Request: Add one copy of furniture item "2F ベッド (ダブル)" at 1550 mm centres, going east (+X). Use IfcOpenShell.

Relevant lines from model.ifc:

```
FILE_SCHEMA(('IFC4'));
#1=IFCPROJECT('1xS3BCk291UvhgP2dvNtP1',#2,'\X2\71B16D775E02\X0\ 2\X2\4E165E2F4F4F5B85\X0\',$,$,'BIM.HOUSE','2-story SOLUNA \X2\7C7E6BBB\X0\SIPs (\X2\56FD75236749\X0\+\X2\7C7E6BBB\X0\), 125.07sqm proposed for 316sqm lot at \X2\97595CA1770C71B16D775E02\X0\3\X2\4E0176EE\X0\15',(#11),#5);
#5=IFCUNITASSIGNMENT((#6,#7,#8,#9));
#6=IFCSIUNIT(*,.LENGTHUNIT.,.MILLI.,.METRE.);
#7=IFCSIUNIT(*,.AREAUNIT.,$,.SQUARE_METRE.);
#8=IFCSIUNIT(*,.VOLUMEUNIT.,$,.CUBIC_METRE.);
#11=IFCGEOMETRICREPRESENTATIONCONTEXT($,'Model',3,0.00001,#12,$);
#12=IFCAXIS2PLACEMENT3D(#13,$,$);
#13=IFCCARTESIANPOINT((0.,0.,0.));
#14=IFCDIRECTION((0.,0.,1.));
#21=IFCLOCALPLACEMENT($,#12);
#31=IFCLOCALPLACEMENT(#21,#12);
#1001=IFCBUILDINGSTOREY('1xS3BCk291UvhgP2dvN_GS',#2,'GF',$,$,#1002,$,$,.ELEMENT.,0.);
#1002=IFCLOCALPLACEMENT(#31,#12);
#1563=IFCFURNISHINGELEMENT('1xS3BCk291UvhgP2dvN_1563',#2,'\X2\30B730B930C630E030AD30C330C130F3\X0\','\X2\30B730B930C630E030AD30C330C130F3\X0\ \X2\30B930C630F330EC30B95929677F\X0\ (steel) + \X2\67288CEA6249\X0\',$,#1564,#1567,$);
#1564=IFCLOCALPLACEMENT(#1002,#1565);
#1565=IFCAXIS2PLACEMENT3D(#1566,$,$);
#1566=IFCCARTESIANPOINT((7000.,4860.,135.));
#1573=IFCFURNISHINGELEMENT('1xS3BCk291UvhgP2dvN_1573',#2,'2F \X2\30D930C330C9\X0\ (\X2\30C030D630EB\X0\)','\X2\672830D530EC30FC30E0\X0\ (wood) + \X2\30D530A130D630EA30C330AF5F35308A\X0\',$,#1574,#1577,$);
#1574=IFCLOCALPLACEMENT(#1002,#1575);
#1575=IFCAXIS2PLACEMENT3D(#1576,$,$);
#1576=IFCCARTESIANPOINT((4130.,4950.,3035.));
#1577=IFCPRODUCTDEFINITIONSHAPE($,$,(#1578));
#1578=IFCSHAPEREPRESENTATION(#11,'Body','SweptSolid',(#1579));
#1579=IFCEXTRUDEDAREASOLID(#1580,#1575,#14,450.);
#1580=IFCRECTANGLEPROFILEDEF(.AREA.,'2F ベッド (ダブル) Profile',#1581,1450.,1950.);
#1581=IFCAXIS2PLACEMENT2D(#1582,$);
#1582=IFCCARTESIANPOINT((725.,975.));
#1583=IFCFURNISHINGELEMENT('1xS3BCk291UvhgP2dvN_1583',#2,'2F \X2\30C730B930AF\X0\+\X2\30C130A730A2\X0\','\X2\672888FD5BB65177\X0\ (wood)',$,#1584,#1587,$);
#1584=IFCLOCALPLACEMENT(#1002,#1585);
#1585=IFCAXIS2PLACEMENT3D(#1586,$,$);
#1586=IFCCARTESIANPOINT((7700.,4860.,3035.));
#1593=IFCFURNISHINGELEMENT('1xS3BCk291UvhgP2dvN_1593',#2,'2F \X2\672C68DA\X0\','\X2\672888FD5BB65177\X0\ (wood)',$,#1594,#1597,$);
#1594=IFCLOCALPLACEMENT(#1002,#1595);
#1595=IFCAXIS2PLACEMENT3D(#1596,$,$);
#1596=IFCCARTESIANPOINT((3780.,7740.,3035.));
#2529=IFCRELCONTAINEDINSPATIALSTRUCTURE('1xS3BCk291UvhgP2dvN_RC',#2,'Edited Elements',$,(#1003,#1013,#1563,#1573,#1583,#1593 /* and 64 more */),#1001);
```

```python
import numpy as np
import ifcopenshell
import ifcopenshell.api.geometry
import ifcopenshell.api.root
import ifcopenshell.util.element
import ifcopenshell.util.placement
import ifcopenshell.util.unit

model = ifcopenshell.open("model.ifc")
unit_scale = ifcopenshell.util.unit.calculate_unit_scale(model)


def reuse_history(source, copy):
    """copy_class also copies each property set's owner history, people and application; keep the originals."""
    for rel in copy.IsDefinedBy:
        if rel.is_a("IfcRelDefinesByProperties") and (history := rel.RelatingPropertyDefinition.OwnerHistory):
            rel.RelatingPropertyDefinition.OwnerHistory = source.OwnerHistory
            ifcopenshell.util.element.remove_deep2(model, history)


source = model.by_id(1573)
base = ifcopenshell.util.placement.get_local_placement(source.ObjectPlacement)
step = np.array([1.0, 0.0, 0.0]) * 1.55 / unit_scale

for i in range(1, 2):
    copy = ifcopenshell.api.root.copy_class(model, product=source)
    copy.Representation = ifcopenshell.util.element.copy_deep(
        model, source.Representation, exclude=["IfcGeometricRepresentationContext", "IfcRepresentationMap"]
    )
    reuse_history(source, copy)
    matrix = base.copy()
    matrix[:3, 3] += i * step
    print("added at", matrix[:3, 3].round(3) + 0.0)
    ifcopenshell.api.geometry.edit_object_placement(model, product=copy, matrix=matrix, is_si=False)

model.write("model_edited.ifc")
```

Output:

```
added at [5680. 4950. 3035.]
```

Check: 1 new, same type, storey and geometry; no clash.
